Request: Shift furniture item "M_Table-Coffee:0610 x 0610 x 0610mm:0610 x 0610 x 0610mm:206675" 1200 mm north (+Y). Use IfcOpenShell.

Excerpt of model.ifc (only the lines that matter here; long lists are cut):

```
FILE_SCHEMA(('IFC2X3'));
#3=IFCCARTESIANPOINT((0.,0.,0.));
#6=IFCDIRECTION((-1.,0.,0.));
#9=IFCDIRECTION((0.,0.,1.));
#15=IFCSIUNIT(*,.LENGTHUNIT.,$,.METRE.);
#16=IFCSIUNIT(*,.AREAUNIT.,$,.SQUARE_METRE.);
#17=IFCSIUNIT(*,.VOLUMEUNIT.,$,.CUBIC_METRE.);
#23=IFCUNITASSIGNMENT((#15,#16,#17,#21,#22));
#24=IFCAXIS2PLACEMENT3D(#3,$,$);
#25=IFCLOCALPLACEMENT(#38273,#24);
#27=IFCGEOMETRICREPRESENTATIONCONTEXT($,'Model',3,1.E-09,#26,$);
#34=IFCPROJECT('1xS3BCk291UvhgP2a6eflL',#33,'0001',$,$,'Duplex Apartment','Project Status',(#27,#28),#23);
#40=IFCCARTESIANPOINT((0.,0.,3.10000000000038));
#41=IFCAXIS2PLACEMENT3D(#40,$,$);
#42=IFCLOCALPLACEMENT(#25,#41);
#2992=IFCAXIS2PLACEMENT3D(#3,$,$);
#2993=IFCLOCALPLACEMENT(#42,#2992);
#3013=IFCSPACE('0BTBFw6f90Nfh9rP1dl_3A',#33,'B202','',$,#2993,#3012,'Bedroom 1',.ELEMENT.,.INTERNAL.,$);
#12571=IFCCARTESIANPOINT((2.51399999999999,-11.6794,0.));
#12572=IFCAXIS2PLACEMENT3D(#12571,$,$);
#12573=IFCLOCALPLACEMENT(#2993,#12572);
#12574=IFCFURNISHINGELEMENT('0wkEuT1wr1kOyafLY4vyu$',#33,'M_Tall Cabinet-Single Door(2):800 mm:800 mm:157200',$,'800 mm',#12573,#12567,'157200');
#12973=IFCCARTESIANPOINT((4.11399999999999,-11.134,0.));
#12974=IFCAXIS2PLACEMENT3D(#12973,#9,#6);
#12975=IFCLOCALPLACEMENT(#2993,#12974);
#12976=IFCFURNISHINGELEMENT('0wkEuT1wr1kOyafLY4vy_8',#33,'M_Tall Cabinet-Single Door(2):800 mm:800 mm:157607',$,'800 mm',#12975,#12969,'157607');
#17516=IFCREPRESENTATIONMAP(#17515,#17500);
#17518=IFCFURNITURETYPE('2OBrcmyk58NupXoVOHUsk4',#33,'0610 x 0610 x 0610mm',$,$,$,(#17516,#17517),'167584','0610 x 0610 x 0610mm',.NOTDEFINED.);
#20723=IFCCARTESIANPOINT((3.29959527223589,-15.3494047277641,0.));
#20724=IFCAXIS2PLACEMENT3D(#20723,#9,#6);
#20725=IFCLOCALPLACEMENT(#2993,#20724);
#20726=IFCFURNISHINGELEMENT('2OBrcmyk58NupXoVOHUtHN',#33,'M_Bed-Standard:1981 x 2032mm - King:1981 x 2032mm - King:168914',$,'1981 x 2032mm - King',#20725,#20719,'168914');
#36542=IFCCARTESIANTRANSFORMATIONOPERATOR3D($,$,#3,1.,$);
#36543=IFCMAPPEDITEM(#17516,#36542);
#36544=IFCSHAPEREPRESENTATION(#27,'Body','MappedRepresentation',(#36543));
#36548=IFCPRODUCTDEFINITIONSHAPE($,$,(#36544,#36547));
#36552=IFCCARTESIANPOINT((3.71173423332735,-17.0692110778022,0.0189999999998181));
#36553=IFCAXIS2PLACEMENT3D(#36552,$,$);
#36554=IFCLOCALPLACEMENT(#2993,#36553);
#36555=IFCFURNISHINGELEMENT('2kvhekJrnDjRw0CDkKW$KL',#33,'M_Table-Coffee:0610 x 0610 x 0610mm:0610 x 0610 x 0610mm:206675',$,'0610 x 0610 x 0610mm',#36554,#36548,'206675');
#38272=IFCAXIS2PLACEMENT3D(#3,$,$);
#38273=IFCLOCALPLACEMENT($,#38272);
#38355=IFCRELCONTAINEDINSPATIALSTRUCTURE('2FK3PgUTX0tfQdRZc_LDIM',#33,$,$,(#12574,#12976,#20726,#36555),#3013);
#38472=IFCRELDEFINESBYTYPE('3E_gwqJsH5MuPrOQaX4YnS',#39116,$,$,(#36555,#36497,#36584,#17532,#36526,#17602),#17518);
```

```python
import ifcopenshell
import ifcopenshell.api.geometry
import ifcopenshell.util.placement
import ifcopenshell.util.unit

model = ifcopenshell.open("model.ifc")
unit_scale = ifcopenshell.util.unit.calculate_unit_scale(model)

item = model.by_id(36555)
matrix = ifcopenshell.util.placement.get_local_placement(item.ObjectPlacement)
matrix[1, 3] += 1.2 / unit_scale
ifcopenshell.api.geometry.edit_object_placement(model, product=item, matrix=matrix, is_si=False)

print(ifcopenshell.util.placement.get_local_placement(item.ObjectPlacement).round(3) + 0.0)

model.write("model_edited.ifc")
```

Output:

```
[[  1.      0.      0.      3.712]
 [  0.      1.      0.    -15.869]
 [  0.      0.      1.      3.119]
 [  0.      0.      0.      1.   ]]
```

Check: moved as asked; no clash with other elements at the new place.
